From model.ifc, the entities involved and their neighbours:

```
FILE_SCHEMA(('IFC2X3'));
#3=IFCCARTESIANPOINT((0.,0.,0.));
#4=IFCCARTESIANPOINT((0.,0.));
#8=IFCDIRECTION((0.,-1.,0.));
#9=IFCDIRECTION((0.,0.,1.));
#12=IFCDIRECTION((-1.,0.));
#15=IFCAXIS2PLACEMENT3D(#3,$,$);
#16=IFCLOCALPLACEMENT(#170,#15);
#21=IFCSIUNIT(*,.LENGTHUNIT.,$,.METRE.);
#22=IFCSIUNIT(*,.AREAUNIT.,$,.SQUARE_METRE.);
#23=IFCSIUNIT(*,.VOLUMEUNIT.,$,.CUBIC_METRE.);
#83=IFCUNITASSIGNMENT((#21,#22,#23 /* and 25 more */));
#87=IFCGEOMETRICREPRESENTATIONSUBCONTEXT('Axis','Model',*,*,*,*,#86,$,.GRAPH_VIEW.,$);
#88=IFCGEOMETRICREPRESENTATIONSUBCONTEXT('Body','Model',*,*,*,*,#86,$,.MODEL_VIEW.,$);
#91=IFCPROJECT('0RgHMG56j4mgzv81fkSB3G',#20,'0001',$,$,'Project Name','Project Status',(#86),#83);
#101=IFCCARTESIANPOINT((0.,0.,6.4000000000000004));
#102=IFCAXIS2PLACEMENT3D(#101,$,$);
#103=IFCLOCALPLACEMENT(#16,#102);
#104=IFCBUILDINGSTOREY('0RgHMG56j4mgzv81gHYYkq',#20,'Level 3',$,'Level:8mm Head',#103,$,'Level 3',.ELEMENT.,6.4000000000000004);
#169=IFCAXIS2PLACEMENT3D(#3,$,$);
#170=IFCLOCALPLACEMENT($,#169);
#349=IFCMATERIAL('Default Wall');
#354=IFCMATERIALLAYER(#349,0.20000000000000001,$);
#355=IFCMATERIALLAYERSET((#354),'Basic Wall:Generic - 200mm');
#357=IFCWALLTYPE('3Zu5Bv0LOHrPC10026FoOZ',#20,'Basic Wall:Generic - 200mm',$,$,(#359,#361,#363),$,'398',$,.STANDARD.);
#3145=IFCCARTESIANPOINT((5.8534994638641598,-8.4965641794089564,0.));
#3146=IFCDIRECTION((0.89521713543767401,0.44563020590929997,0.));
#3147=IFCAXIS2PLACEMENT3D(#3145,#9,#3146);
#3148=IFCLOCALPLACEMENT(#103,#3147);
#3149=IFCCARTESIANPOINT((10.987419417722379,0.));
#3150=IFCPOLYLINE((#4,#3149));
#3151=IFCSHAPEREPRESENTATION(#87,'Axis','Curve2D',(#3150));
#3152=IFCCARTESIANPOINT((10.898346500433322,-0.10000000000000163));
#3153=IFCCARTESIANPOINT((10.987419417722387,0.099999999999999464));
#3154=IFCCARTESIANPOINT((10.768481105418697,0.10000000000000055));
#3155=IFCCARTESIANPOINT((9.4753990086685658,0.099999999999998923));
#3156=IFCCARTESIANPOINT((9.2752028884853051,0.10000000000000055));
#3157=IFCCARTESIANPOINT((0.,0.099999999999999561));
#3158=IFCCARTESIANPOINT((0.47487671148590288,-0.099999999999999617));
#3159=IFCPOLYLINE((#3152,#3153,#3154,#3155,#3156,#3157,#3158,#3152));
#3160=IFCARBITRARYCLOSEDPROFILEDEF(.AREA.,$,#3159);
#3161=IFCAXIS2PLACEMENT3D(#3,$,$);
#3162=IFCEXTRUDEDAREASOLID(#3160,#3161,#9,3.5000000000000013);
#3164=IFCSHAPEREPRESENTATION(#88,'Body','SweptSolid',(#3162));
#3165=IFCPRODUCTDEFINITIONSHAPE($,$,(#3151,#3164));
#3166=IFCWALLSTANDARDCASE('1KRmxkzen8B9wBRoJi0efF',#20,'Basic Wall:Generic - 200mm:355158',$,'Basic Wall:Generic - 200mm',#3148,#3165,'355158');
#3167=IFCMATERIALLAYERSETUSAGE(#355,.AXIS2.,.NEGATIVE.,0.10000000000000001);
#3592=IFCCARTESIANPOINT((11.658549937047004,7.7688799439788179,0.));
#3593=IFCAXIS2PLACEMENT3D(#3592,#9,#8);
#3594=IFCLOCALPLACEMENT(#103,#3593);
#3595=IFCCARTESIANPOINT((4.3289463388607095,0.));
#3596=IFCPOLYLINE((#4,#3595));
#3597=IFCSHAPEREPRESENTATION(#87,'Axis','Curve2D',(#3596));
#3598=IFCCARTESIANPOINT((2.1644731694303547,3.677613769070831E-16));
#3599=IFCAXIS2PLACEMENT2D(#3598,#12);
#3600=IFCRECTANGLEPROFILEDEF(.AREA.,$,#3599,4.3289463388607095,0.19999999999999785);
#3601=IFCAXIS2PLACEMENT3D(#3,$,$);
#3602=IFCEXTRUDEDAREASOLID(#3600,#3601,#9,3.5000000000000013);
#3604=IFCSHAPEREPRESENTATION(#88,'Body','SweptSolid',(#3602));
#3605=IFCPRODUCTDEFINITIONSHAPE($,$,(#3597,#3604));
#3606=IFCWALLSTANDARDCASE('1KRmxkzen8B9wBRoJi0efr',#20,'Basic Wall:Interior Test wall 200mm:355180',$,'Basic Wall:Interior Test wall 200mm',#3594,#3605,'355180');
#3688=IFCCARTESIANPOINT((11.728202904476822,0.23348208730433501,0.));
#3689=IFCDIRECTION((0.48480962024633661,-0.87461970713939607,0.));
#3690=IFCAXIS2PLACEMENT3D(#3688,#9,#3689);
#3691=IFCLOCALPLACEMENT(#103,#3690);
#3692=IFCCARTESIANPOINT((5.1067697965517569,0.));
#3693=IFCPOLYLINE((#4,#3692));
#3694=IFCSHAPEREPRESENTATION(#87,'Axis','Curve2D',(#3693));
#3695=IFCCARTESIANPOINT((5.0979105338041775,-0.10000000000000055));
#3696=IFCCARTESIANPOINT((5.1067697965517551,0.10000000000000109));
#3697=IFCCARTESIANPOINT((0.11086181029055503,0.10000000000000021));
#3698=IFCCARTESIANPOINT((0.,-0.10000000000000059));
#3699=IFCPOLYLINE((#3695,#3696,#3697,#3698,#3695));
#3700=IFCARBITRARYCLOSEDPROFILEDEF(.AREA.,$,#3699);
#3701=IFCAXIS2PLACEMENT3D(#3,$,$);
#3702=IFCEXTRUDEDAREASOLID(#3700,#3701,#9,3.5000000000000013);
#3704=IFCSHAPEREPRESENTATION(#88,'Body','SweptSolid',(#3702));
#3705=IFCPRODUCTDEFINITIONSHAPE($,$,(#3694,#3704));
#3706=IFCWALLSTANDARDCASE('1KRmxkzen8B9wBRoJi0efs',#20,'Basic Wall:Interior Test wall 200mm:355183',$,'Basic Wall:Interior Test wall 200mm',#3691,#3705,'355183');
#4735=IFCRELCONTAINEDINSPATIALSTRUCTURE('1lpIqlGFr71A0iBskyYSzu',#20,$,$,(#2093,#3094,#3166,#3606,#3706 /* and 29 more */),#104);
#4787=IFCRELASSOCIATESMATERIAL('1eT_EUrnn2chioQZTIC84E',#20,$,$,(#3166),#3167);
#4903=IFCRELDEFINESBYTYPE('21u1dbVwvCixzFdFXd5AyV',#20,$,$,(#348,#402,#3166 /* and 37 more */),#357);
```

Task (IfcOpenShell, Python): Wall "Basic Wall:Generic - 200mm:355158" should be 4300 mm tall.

```python
import ifcopenshell
import ifcopenshell.geom
import ifcopenshell.util.representation
import ifcopenshell.util.shape

model = ifcopenshell.open("model.ifc")
settings = ifcopenshell.geom.settings()


def volume(element):
    """Net volume in cubic metres, openings subtracted."""
    shape = ifcopenshell.geom.create_shape(settings, element)
    return ifcopenshell.util.shape.get_volume(shape.geometry)


wall = model.by_id(3166)
before = volume(wall)

body = ifcopenshell.util.representation.get_representation(wall, "Model", "Body")
solid = body.Items[0]
old_height = solid.Depth
solid.Depth = 4.3
after = volume(wall)

print(f"height {old_height:g} -> {solid.Depth:g}, volume {before:.3f} -> {after:.3f} m3")

model.write("model_updated.ifc")
```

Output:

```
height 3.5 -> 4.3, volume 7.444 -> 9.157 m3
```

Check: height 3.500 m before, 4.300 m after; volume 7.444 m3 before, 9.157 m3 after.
